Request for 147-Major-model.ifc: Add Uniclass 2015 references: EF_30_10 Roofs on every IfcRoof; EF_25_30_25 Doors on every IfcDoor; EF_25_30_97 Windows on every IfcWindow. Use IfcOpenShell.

First a look at what the model holds.

```python
import ifcopenshell

model = ifcopenshell.open("147-Major-model.ifc")
print(model.schema)
print("classifications:", [c.Name for c in model.by_type("IfcClassification")])
for ifc_class in ("IfcDoor", "IfcRoof", "IfcStair", "IfcWall", "IfcWindow"):
    print(ifc_class, len(model.by_type(ifc_class)))
```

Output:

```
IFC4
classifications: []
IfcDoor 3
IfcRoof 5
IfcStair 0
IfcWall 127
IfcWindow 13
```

```python
import ifcopenshell
import ifcopenshell.api.classification

model = ifcopenshell.open("147-Major-model.ifc")

system = ifcopenshell.api.classification.add_classification(model, classification="Uniclass 2015")

codes = {
    "IfcRoof": ("EF_30_10", "Roofs"),
    "IfcDoor": ("EF_25_30_25", "Doors"),
    "IfcWindow": ("EF_25_30_97", "Windows"),
}
for ifc_class, (code, name) in codes.items():
    products = model.by_type(ifc_class)
    ifcopenshell.api.classification.add_reference(
        model, products=products, classification=system, identification=code, name=name
    )
    print(code, len(products))

model.write("147-Major-model_v2.ifc")
```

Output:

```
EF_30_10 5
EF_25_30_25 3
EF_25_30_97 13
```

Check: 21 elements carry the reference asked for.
